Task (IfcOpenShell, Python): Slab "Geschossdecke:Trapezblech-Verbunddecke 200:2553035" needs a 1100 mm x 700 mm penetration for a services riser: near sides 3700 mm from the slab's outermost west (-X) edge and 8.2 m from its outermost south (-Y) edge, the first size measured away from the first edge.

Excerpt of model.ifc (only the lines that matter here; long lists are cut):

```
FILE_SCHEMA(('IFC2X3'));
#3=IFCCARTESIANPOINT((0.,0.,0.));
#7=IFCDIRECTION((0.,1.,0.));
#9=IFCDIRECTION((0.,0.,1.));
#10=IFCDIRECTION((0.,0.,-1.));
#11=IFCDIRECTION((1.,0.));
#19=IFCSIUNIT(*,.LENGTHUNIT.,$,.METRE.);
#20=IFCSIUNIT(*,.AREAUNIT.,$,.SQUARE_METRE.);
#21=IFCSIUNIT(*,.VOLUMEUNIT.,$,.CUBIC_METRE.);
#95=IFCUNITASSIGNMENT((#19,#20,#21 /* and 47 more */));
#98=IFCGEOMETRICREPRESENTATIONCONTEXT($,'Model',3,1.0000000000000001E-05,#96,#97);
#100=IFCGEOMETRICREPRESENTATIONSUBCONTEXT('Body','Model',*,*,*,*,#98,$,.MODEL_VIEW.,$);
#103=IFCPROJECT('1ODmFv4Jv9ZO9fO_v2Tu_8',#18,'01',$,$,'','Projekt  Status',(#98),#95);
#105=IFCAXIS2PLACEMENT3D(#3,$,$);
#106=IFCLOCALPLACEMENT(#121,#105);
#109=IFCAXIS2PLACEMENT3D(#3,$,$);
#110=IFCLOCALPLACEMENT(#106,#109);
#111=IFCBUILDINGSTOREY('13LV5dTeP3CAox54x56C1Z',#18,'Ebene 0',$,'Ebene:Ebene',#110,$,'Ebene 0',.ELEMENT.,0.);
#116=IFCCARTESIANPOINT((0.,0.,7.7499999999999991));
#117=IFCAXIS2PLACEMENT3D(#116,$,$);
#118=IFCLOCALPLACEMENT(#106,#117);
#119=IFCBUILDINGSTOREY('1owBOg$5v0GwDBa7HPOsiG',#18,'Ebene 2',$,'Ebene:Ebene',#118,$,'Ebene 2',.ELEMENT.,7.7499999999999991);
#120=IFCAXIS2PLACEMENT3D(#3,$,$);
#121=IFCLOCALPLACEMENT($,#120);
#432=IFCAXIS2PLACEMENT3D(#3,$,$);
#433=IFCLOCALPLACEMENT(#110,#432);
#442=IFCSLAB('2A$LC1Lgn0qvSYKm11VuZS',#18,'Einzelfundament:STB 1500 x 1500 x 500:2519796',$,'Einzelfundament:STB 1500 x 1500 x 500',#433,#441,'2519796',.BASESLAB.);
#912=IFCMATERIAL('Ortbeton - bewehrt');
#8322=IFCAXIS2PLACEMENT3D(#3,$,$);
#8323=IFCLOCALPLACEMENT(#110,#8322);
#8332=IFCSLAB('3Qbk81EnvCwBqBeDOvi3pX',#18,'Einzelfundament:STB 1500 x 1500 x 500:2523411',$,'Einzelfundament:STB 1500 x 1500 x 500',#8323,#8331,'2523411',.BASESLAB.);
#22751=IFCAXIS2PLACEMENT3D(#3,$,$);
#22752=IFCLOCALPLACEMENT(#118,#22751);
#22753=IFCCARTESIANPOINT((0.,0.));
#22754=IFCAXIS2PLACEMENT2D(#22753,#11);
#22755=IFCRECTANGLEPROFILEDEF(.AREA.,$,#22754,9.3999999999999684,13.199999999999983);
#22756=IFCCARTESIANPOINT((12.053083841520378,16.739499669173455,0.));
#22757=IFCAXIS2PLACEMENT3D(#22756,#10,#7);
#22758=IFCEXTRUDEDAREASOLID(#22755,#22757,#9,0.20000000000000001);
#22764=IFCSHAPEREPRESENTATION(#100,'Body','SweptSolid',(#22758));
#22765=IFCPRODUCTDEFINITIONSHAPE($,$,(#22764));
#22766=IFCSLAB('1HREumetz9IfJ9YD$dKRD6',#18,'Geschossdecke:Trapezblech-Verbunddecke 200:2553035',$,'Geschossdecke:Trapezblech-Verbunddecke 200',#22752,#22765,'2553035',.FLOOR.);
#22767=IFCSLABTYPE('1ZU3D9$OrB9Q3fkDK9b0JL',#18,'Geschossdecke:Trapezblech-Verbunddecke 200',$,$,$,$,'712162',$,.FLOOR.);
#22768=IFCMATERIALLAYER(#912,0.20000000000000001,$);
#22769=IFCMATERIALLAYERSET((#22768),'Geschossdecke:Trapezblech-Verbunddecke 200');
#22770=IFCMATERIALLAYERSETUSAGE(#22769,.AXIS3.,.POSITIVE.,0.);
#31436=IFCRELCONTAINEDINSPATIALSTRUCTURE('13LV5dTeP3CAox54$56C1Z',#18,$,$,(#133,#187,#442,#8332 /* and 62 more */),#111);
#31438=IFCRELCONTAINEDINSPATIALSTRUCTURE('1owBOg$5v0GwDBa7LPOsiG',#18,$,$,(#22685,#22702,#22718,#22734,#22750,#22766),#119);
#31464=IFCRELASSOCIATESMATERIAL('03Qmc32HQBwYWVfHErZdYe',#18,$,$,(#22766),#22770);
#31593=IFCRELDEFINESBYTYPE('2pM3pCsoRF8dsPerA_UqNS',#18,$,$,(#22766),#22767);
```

```python
import numpy as np
import ifcopenshell
import ifcopenshell.api.feature
import ifcopenshell.api.geometry
import ifcopenshell.api.root
import ifcopenshell.geom
import ifcopenshell.util.placement
import ifcopenshell.util.representation
import ifcopenshell.util.shape
import ifcopenshell.util.unit

model = ifcopenshell.open("model.ifc")
unit_scale = ifcopenshell.util.unit.calculate_unit_scale(model)
settings = ifcopenshell.geom.settings()


def volume(element):
    """Net volume in cubic metres, openings subtracted."""
    shape = ifcopenshell.geom.create_shape(settings, element)
    return ifcopenshell.util.shape.get_volume(shape.geometry)


slab = model.by_guid("1HREumetz9IfJ9YD$dKRD6")
before = volume(slab)

# Extent in the slab's own axes, in metres. The edges named are its -X and -Y sides.
slab_shape = ifcopenshell.geom.create_shape(settings, slab)
vertices = ifcopenshell.util.shape.get_vertices(slab_shape.geometry)
x_min, y_min, bottom = vertices.min(axis=0)
top = vertices[:, 2].max()

opening = ifcopenshell.api.root.create_entity(model, ifc_class="IfcOpeningElement", name="Services riser opening")
context = ifcopenshell.util.representation.get_context(model, "Model", "Body", "MODEL_VIEW")
width, depth = 1.1, 0.7
outline = [(0.0, 0.0), (width, 0.0), (width, depth), (0.0, depth), (0.0, 0.0)]
# Overshoot both faces by 50 mm so the cut is clean.
shape = ifcopenshell.api.geometry.add_slab_representation(
    model, context=context, depth=top - bottom + 0.1, polyline=outline
)
ifcopenshell.api.geometry.assign_representation(model, product=opening, representation=shape)

matrix = ifcopenshell.util.placement.get_local_placement(slab.ObjectPlacement)
matrix[:, 3] = matrix @ np.append(np.array([x_min + 3.7, y_min + 8.2, bottom - 0.05]) / unit_scale, 1.0)
ifcopenshell.api.geometry.edit_object_placement(model, product=opening, matrix=matrix, is_si=False)
ifcopenshell.api.feature.add_feature(model, feature=opening, element=slab)

after = volume(slab)

print(f"slab volume {before:.3f} -> {after:.3f} m3")

model.write("model_updated.ifc")
```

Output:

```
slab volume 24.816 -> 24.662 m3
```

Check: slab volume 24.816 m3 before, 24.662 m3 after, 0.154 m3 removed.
